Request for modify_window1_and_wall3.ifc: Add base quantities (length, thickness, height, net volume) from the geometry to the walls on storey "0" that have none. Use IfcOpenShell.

First a look at what the model holds.

```python
import ifcopenshell
import ifcopenshell.util.element
import ifcopenshell.util.unit

model = ifcopenshell.open("modify_window1_and_wall3.ifc")
print(model.schema)
for unit_type in ("LENGTHUNIT", "AREAUNIT", "VOLUMEUNIT"):
    print(unit_type, ifcopenshell.util.unit.calculate_unit_scale(model, unit_type))
storey = next(s for s in model.by_type("IfcBuildingStorey") if s.Name == "0")
walls = [e for e in ifcopenshell.util.element.get_decomposition(storey) if e.is_a("IfcWall")]
for e in sorted(walls, key=lambda e: e.id()):
    print(e.id(), e.is_a(), e.Name, list(ifcopenshell.util.element.get_psets(e, qtos_only=True)), sep=" | ")
```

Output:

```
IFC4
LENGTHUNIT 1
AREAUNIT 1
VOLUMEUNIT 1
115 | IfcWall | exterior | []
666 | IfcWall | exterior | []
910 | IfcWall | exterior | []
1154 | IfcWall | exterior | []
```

```python
import ifcopenshell
import ifcopenshell.api.pset
import ifcopenshell.geom
import ifcopenshell.util.element
import ifcopenshell.util.shape
import ifcopenshell.util.unit

model = ifcopenshell.open("modify_window1_and_wall3.ifc")
unit_scale = ifcopenshell.util.unit.calculate_unit_scale(model)
volume_scale = ifcopenshell.util.unit.calculate_unit_scale(model, "VOLUMEUNIT")
settings = ifcopenshell.geom.settings()

storey = next(s for s in model.by_type("IfcBuildingStorey") if s.Name == "0")
walls = [e for e in ifcopenshell.util.element.get_decomposition(storey) if e.is_a("IfcWall")]

for e in sorted(walls, key=lambda e: e.id()):
    if ifcopenshell.util.element.get_psets(e, qtos_only=True, should_inherit=False):
        continue
    # Geometry comes back in metres, in the element's own axes.
    shape = ifcopenshell.geom.create_shape(settings, e)
    values = {
        "Length": ifcopenshell.util.shape.get_x(shape.geometry) / unit_scale,
        "Width": ifcopenshell.util.shape.get_y(shape.geometry) / unit_scale,
        "Height": ifcopenshell.util.shape.get_z(shape.geometry) / unit_scale,
        "NetVolume": ifcopenshell.util.shape.get_volume(shape.geometry) / volume_scale,
    }
    qto = ifcopenshell.api.pset.add_qto(model, product=e, name="Qto_WallBaseQuantities")
    ifcopenshell.api.pset.edit_qto(model, qto=qto, properties=values)
    print(e.id(), {k: round(v, 3) for k, v in values.items()})

model.write("modify_window1_and_wall3_updated.ifc")
```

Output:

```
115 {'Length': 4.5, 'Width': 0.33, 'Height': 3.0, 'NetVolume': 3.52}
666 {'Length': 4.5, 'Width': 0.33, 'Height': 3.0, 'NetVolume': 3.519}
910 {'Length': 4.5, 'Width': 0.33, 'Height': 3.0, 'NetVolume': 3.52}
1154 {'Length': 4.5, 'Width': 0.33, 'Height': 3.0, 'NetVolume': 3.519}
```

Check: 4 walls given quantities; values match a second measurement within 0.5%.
